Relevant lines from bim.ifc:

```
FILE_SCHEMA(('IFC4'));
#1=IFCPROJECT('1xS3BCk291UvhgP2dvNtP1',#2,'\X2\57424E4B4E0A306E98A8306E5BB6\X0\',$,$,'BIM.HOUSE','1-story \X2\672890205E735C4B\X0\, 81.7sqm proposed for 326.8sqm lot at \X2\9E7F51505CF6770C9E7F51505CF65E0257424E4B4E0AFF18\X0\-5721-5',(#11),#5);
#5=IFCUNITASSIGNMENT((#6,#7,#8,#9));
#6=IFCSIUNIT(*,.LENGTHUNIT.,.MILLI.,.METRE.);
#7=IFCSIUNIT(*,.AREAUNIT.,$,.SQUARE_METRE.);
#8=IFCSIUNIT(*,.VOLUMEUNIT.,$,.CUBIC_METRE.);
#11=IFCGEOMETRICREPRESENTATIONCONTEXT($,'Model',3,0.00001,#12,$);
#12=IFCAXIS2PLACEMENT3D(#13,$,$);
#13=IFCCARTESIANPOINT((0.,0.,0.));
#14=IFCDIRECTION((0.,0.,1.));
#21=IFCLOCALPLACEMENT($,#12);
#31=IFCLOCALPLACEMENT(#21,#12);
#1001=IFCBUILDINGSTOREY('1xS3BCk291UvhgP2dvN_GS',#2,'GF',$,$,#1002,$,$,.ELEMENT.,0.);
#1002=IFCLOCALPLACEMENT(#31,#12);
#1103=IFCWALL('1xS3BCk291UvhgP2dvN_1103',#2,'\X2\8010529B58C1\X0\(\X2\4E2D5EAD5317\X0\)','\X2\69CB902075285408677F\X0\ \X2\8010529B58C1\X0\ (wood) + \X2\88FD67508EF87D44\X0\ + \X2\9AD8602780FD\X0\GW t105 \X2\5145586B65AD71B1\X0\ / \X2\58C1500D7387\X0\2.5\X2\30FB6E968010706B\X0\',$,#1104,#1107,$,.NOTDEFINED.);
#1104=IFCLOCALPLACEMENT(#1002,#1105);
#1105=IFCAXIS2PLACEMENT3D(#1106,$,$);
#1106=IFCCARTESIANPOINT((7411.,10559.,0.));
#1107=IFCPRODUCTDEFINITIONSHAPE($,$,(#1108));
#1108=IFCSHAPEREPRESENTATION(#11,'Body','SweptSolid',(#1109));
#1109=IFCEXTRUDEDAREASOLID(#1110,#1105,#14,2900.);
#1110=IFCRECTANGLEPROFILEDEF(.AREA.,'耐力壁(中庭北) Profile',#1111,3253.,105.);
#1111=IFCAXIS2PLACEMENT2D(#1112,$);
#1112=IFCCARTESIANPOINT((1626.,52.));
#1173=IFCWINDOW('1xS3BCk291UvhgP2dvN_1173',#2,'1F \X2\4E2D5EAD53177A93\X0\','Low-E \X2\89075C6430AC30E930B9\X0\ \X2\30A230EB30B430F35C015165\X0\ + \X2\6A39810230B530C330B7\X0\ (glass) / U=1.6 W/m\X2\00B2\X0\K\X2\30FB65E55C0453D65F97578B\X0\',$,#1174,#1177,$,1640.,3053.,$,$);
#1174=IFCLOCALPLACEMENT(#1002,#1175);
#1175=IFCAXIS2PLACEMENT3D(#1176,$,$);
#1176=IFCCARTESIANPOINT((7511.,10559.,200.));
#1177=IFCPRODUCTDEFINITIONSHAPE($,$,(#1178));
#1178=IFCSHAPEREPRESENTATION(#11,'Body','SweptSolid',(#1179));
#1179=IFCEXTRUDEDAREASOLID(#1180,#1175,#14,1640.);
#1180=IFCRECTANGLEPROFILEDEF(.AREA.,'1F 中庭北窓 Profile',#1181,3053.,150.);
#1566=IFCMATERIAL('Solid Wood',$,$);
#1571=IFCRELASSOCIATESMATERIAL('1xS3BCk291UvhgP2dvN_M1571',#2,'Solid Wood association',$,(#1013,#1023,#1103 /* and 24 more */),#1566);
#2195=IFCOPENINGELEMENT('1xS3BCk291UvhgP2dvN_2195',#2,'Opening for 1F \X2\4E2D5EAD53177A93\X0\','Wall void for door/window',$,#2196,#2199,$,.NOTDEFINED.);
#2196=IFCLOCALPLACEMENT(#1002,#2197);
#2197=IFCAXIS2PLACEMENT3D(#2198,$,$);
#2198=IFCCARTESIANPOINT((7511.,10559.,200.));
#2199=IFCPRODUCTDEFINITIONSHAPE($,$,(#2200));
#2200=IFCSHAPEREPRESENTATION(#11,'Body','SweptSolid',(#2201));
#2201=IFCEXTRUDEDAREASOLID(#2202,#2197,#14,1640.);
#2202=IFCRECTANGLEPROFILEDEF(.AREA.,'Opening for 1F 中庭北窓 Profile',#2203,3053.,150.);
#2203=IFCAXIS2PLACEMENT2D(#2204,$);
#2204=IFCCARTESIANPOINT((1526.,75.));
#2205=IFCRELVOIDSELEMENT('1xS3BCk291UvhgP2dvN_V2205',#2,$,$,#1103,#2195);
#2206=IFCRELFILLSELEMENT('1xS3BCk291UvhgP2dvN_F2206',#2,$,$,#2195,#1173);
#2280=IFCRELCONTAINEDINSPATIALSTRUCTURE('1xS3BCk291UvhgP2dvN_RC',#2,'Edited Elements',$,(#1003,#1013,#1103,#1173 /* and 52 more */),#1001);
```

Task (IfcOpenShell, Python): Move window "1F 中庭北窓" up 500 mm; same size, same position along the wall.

```python
import numpy as np
import ifcopenshell
import ifcopenshell.api.geometry
import ifcopenshell.util.placement
import ifcopenshell.util.unit

model = ifcopenshell.open("bim.ifc")
unit_scale = ifcopenshell.util.unit.calculate_unit_scale(model)

window = model.by_id(1173)
opening = window.FillsVoids[0].RelatingOpeningElement
dz = 0.5 / unit_scale

shift = np.array([0.0, 0.0, dz])
# The window is not placed relative to its opening, so move both.
for product in (opening, window):
    matrix = ifcopenshell.util.placement.get_local_placement(product.ObjectPlacement)
    matrix[:3, 3] += shift
    ifcopenshell.api.geometry.edit_object_placement(model, product=product, matrix=matrix, is_si=False)

print(f"moved by {dz * unit_scale:+.3f} m")

model.write("bim_updated.ifc")
```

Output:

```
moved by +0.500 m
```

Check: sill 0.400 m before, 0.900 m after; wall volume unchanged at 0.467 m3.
